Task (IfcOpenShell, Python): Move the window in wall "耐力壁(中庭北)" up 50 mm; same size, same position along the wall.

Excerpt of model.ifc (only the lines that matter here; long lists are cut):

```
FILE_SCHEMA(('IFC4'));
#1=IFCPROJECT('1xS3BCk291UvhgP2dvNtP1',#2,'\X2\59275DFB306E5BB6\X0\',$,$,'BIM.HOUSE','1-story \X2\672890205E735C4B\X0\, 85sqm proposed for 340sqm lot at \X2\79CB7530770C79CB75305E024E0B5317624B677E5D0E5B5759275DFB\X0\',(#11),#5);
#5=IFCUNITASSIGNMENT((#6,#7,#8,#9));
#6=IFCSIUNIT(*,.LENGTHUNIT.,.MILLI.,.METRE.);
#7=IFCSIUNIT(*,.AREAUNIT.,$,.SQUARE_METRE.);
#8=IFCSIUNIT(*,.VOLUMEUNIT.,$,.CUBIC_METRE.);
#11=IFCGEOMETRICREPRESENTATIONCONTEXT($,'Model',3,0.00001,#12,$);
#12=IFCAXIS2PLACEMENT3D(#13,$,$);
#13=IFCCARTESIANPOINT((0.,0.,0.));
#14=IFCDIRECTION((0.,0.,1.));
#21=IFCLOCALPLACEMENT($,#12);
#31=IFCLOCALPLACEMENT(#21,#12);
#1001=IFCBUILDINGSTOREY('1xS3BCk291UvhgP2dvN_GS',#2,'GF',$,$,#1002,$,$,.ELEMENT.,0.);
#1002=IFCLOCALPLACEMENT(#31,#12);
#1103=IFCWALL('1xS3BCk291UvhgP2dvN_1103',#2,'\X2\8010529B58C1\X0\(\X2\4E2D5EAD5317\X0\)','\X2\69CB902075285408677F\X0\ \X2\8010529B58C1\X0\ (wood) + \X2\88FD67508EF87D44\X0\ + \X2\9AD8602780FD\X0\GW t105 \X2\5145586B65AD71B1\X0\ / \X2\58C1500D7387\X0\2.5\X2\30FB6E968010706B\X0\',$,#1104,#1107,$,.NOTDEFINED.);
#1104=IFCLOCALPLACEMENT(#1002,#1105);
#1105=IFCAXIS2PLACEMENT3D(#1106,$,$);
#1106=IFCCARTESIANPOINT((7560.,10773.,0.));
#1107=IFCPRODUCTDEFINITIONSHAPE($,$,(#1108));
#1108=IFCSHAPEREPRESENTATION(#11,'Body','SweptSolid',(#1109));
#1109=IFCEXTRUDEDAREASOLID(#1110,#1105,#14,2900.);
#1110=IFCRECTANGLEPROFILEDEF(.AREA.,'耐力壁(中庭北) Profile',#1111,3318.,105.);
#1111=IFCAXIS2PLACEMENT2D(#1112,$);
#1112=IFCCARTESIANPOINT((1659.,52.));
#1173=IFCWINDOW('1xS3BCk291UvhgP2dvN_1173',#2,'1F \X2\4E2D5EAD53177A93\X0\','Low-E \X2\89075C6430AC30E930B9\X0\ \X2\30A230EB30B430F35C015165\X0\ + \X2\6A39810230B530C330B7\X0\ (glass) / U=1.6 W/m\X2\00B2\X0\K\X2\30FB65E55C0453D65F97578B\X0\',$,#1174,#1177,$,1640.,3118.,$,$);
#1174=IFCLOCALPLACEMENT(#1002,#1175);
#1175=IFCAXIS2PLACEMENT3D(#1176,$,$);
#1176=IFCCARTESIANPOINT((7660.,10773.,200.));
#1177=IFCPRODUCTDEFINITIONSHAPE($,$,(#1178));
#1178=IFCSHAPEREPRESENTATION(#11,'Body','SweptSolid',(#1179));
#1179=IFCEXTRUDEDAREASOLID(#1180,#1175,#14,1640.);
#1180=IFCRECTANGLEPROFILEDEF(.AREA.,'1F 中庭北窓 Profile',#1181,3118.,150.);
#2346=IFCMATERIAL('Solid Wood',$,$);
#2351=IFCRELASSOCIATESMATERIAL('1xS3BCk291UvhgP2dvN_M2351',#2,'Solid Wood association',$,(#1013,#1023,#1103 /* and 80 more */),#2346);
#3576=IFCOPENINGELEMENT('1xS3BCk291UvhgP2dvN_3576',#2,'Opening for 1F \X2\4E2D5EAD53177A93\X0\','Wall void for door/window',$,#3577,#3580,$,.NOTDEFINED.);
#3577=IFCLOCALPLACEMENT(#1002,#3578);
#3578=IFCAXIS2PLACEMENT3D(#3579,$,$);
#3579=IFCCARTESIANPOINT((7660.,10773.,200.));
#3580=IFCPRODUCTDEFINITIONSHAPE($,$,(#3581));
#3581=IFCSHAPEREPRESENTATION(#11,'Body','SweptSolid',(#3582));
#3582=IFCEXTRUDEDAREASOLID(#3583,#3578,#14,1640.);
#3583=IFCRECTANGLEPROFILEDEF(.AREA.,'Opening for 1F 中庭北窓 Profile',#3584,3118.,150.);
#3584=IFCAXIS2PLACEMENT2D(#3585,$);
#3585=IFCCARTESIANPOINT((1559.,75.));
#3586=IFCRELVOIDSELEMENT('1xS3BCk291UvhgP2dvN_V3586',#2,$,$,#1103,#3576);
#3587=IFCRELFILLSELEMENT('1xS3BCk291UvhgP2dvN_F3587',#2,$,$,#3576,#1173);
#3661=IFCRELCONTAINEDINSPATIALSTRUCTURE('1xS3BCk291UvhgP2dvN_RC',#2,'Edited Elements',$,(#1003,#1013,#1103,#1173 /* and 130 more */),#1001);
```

```python
import numpy as np
import ifcopenshell
import ifcopenshell.api.geometry
import ifcopenshell.util.placement
import ifcopenshell.util.unit

model = ifcopenshell.open("model.ifc")
unit_scale = ifcopenshell.util.unit.calculate_unit_scale(model)

window = model.by_guid("1xS3BCk291UvhgP2dvN_1173")
opening = window.FillsVoids[0].RelatingOpeningElement
dz = 0.05 / unit_scale

shift = np.array([0.0, 0.0, dz])
# The window is not placed relative to its opening, so move both.
for product in (opening, window):
    matrix = ifcopenshell.util.placement.get_local_placement(product.ObjectPlacement)
    matrix[:3, 3] += shift
    ifcopenshell.api.geometry.edit_object_placement(model, product=product, matrix=matrix, is_si=False)

print(f"moved by {dz * unit_scale:+.3f} m")

model.write("model_updated.ifc")
```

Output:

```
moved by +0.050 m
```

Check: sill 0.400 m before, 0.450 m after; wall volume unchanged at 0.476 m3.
